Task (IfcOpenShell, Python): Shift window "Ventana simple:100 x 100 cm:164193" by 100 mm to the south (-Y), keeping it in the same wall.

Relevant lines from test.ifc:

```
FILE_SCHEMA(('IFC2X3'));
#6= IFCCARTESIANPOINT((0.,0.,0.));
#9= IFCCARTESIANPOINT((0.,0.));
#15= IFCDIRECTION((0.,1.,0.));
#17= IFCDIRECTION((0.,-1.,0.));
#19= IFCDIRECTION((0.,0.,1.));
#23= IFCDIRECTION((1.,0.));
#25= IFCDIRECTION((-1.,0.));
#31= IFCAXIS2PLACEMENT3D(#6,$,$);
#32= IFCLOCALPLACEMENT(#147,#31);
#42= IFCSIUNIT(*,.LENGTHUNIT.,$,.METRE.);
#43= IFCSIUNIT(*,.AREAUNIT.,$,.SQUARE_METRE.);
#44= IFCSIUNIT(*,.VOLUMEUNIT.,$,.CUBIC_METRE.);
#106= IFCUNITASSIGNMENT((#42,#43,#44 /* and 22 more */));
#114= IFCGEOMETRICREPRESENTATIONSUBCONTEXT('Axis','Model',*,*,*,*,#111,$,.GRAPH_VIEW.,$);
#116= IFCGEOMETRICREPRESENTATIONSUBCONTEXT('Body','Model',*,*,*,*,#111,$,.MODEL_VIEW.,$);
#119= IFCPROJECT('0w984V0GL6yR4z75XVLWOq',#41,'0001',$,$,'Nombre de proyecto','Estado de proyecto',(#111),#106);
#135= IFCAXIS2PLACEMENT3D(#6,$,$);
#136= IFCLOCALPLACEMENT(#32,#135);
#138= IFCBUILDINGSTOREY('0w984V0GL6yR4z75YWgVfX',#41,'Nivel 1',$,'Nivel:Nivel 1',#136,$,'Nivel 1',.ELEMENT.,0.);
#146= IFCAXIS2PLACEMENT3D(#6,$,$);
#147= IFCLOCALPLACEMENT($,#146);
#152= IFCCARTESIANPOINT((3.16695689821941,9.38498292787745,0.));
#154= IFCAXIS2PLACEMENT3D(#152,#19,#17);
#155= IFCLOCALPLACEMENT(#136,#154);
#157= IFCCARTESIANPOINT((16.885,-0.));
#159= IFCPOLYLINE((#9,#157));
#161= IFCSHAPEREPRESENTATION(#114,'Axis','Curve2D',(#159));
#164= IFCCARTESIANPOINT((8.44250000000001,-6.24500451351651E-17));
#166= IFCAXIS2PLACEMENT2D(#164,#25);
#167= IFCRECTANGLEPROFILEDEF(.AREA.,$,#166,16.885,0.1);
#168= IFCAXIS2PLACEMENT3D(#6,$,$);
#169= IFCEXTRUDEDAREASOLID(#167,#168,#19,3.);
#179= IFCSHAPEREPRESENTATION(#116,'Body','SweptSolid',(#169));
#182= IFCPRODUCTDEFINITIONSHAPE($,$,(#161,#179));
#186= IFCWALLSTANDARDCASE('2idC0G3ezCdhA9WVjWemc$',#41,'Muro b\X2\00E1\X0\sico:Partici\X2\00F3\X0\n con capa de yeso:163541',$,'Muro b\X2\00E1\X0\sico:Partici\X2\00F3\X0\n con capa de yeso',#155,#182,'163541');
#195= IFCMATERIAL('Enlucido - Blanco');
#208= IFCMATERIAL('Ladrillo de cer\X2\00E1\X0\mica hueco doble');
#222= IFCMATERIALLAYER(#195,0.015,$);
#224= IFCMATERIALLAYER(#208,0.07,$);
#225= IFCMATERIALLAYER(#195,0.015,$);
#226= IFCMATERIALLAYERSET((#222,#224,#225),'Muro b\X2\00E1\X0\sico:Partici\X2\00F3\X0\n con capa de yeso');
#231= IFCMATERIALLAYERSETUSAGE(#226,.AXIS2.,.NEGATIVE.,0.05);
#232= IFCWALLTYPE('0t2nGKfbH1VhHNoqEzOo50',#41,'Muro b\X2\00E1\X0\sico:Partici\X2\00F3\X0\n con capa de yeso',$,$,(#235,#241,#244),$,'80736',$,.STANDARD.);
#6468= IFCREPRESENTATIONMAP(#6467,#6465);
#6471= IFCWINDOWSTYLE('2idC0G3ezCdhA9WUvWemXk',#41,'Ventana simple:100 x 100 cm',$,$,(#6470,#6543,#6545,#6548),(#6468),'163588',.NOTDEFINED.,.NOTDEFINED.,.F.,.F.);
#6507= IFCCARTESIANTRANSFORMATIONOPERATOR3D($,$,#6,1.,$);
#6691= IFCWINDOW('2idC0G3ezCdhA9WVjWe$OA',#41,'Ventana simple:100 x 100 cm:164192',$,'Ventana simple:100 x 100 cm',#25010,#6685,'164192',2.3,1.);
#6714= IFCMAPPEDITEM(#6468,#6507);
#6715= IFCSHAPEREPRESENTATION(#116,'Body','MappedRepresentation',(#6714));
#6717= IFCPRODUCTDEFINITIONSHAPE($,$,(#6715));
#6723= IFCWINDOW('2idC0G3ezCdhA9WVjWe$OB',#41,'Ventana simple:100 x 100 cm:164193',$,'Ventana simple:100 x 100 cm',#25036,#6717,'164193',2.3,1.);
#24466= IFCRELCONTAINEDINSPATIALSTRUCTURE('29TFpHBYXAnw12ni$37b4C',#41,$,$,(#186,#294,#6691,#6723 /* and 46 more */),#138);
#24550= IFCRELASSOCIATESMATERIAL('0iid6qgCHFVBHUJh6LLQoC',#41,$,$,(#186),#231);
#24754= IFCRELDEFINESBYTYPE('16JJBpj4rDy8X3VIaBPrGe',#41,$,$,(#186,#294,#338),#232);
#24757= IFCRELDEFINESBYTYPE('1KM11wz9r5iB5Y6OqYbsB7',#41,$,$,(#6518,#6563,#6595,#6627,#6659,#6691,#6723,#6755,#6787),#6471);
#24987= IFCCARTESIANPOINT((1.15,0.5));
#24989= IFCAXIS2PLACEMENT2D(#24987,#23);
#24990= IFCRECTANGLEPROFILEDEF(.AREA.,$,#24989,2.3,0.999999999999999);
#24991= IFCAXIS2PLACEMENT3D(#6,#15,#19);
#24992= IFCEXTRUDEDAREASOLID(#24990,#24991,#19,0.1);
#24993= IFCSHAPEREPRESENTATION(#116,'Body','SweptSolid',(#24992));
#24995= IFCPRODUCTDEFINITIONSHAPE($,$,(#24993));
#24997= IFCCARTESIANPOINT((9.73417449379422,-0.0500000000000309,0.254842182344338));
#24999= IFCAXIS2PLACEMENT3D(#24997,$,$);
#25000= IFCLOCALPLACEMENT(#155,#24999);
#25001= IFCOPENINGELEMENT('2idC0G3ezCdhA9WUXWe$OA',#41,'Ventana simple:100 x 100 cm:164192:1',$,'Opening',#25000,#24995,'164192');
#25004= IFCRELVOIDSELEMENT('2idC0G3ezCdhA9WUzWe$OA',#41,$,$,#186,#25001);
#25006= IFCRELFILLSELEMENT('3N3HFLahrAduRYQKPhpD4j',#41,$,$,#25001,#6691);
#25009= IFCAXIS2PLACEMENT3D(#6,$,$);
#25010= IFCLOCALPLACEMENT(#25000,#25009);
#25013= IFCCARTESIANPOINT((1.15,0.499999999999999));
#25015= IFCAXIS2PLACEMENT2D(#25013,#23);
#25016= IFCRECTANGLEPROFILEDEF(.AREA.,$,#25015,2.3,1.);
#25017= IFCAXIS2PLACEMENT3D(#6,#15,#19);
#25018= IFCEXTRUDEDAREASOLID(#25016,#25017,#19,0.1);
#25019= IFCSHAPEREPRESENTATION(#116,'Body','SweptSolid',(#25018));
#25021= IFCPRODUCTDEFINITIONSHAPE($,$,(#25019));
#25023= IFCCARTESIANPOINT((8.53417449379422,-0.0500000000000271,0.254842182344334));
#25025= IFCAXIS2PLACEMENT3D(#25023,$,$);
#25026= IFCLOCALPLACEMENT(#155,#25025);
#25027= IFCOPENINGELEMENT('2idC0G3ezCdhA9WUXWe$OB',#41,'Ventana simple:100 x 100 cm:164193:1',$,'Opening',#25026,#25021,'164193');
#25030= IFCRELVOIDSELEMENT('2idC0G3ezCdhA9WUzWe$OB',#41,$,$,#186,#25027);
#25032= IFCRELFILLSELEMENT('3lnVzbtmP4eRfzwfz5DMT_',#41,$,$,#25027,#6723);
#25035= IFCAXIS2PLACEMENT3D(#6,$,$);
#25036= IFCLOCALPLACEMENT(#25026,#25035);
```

```python
import ifcopenshell
import ifcopenshell.api.geometry
import ifcopenshell.util.placement
import ifcopenshell.util.unit

model = ifcopenshell.open("test.ifc")
unit_scale = ifcopenshell.util.unit.calculate_unit_scale(model)

window = model.by_guid("2idC0G3ezCdhA9WVjWe$OB")
opening = window.FillsVoids[0].RelatingOpeningElement
wall = opening.VoidsElements[0].RelatingBuildingElement

wall_matrix = ifcopenshell.util.placement.get_local_placement(wall.ObjectPlacement)
shift = wall_matrix[:3, 0] * 0.1 / unit_scale
before = ifcopenshell.util.placement.get_local_placement(window.ObjectPlacement)[:3, 3].copy()

# The window is placed relative to its opening, so it follows when the opening moves.
matrix = ifcopenshell.util.placement.get_local_placement(opening.ObjectPlacement)
matrix[:3, 3] += shift
ifcopenshell.api.geometry.edit_object_placement(
    model, product=opening, matrix=matrix, is_si=False, should_transform_children=True
)

after = ifcopenshell.util.placement.get_local_placement(window.ObjectPlacement)[:3, 3]
print("window moved by", (after - before).round(3) + 0.0)

model.write("test_v2.ifc")
```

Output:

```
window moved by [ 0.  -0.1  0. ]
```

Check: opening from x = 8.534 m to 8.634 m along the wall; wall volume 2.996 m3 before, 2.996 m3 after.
